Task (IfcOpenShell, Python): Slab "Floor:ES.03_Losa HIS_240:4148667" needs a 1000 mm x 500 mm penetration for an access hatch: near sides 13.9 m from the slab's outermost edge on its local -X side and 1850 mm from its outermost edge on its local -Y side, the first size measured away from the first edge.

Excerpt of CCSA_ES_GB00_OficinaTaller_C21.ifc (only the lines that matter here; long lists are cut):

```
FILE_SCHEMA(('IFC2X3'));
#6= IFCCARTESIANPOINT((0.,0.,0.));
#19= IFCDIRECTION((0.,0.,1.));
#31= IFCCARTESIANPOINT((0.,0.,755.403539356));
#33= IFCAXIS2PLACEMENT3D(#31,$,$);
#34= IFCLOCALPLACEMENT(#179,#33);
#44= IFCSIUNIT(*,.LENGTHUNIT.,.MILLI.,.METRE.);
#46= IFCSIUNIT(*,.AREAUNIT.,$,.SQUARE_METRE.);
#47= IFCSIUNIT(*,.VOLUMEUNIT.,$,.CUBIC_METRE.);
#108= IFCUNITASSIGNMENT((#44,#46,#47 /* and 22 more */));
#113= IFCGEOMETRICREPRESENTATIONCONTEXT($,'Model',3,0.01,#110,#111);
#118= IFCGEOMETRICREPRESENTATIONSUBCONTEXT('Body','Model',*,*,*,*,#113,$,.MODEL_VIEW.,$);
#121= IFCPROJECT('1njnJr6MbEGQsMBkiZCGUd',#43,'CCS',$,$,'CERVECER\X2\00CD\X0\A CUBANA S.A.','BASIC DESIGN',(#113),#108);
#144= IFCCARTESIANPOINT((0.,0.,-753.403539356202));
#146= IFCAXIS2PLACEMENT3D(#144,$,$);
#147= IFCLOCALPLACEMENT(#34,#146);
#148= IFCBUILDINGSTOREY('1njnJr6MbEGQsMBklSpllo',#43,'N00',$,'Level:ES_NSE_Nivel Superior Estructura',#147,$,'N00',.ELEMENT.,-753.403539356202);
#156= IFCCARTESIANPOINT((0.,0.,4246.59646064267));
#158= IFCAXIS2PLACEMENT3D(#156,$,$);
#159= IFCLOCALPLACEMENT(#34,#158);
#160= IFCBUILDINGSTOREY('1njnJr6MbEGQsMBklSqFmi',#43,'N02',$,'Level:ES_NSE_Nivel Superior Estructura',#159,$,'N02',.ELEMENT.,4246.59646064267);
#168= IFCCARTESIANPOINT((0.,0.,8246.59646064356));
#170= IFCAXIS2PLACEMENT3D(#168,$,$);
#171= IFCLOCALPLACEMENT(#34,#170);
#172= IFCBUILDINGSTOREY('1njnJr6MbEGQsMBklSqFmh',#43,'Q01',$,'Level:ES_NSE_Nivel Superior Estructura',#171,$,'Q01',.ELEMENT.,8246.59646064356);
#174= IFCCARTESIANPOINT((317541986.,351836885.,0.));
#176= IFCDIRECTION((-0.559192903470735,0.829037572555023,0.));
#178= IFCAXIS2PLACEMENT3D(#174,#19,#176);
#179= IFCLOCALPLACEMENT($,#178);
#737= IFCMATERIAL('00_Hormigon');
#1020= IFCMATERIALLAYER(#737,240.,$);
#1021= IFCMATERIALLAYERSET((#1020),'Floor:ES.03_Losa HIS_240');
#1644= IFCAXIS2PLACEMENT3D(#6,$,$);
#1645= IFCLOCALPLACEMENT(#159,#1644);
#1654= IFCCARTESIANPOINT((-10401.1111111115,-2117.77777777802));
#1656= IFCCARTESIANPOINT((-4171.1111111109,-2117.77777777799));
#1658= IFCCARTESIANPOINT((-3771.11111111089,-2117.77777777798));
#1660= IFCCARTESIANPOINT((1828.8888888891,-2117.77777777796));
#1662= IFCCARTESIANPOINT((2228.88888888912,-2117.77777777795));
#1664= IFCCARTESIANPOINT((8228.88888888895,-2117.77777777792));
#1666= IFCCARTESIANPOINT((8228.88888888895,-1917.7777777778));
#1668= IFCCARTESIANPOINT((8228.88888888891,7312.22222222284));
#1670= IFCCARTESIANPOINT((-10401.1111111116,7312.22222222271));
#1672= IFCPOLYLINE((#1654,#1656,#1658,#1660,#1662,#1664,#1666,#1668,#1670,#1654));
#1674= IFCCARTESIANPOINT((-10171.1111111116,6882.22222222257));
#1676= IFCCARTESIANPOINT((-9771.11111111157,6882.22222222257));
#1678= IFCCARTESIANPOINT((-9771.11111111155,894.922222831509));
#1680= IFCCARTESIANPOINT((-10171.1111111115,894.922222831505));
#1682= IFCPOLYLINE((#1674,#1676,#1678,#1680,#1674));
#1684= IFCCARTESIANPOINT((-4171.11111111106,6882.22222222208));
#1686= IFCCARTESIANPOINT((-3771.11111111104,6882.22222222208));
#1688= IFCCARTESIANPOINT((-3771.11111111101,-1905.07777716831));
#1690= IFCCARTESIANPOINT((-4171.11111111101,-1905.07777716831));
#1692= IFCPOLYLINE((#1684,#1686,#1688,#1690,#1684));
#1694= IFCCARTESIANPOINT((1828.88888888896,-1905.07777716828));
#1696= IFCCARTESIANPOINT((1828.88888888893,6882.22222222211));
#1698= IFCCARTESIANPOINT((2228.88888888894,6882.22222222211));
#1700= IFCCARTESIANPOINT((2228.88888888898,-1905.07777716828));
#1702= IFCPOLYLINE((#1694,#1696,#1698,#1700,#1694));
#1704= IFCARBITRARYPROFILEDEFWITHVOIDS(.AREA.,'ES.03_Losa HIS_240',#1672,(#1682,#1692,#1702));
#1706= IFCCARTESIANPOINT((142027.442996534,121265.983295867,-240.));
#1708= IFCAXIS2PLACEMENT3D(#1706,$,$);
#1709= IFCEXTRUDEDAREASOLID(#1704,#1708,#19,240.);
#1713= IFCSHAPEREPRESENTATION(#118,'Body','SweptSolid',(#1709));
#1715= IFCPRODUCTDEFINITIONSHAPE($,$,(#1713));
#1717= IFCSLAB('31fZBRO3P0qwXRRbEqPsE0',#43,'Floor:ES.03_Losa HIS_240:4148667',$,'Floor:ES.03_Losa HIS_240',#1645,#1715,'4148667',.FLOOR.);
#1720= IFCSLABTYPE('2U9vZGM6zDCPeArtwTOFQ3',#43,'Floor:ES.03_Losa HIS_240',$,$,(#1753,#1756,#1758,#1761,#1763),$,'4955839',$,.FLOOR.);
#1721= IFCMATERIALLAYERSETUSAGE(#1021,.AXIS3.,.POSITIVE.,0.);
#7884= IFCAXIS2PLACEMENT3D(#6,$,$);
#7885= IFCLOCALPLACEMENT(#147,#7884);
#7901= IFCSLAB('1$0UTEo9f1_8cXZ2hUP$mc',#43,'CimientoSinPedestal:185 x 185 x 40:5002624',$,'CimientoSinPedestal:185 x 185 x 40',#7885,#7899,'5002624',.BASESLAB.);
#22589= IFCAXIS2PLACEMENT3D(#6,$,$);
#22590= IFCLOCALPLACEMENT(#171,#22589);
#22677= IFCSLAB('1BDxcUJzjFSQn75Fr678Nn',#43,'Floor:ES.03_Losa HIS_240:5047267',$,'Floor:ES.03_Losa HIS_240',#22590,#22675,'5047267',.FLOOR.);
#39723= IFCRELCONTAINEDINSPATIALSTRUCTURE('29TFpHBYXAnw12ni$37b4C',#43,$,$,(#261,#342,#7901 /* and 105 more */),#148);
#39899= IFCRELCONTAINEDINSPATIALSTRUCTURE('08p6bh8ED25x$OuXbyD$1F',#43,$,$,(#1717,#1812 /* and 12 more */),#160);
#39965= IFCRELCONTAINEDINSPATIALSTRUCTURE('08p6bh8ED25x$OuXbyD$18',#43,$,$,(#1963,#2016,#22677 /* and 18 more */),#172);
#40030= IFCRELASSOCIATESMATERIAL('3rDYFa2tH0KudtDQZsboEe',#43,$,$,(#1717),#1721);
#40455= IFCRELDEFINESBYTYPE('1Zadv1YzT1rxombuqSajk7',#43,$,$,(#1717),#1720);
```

```python
import numpy as np
import ifcopenshell
import ifcopenshell.api.feature
import ifcopenshell.api.geometry
import ifcopenshell.api.root
import ifcopenshell.geom
import ifcopenshell.util.placement
import ifcopenshell.util.representation
import ifcopenshell.util.shape
import ifcopenshell.util.unit

model = ifcopenshell.open("CCSA_ES_GB00_OficinaTaller_C21.ifc")
unit_scale = ifcopenshell.util.unit.calculate_unit_scale(model)
settings = ifcopenshell.geom.settings()


def volume(element):
    """Net volume in cubic metres, openings subtracted."""
    shape = ifcopenshell.geom.create_shape(settings, element)
    return ifcopenshell.util.shape.get_volume(shape.geometry)


slab = model.by_id(1717)
before = volume(slab)

# Extent in the slab's own axes, in metres. The edges named are its -X and -Y sides.
slab_shape = ifcopenshell.geom.create_shape(settings, slab)
vertices = ifcopenshell.util.shape.get_vertices(slab_shape.geometry)
x_min, y_min, bottom = vertices.min(axis=0)
top = vertices[:, 2].max()

opening = ifcopenshell.api.root.create_entity(model, ifc_class="IfcOpeningElement", name="Access hatch opening")
context = ifcopenshell.util.representation.get_context(model, "Model", "Body", "MODEL_VIEW")
width, depth = 1, 0.5
outline = [(0.0, 0.0), (width, 0.0), (width, depth), (0.0, depth), (0.0, 0.0)]
# Overshoot both faces by 50 mm so the cut is clean.
shape = ifcopenshell.api.geometry.add_slab_representation(
    model, context=context, depth=top - bottom + 0.1, polyline=outline
)
ifcopenshell.api.geometry.assign_representation(model, product=opening, representation=shape)

matrix = ifcopenshell.util.placement.get_local_placement(slab.ObjectPlacement)
matrix[:, 3] = matrix @ np.append(np.array([x_min + 13.9, y_min + 1.85, bottom - 0.05]) / unit_scale, 1.0)
ifcopenshell.api.geometry.edit_object_placement(model, product=opening, matrix=matrix, is_si=False)
ifcopenshell.api.feature.add_feature(model, feature=opening, element=slab)

after = volume(slab)

print(f"slab volume {before:.3f} -> {after:.3f} m3")

model.write("CCSA_ES_GB00_OficinaTaller_C21_edited.ifc")
```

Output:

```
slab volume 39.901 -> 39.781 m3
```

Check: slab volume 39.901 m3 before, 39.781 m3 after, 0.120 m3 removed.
